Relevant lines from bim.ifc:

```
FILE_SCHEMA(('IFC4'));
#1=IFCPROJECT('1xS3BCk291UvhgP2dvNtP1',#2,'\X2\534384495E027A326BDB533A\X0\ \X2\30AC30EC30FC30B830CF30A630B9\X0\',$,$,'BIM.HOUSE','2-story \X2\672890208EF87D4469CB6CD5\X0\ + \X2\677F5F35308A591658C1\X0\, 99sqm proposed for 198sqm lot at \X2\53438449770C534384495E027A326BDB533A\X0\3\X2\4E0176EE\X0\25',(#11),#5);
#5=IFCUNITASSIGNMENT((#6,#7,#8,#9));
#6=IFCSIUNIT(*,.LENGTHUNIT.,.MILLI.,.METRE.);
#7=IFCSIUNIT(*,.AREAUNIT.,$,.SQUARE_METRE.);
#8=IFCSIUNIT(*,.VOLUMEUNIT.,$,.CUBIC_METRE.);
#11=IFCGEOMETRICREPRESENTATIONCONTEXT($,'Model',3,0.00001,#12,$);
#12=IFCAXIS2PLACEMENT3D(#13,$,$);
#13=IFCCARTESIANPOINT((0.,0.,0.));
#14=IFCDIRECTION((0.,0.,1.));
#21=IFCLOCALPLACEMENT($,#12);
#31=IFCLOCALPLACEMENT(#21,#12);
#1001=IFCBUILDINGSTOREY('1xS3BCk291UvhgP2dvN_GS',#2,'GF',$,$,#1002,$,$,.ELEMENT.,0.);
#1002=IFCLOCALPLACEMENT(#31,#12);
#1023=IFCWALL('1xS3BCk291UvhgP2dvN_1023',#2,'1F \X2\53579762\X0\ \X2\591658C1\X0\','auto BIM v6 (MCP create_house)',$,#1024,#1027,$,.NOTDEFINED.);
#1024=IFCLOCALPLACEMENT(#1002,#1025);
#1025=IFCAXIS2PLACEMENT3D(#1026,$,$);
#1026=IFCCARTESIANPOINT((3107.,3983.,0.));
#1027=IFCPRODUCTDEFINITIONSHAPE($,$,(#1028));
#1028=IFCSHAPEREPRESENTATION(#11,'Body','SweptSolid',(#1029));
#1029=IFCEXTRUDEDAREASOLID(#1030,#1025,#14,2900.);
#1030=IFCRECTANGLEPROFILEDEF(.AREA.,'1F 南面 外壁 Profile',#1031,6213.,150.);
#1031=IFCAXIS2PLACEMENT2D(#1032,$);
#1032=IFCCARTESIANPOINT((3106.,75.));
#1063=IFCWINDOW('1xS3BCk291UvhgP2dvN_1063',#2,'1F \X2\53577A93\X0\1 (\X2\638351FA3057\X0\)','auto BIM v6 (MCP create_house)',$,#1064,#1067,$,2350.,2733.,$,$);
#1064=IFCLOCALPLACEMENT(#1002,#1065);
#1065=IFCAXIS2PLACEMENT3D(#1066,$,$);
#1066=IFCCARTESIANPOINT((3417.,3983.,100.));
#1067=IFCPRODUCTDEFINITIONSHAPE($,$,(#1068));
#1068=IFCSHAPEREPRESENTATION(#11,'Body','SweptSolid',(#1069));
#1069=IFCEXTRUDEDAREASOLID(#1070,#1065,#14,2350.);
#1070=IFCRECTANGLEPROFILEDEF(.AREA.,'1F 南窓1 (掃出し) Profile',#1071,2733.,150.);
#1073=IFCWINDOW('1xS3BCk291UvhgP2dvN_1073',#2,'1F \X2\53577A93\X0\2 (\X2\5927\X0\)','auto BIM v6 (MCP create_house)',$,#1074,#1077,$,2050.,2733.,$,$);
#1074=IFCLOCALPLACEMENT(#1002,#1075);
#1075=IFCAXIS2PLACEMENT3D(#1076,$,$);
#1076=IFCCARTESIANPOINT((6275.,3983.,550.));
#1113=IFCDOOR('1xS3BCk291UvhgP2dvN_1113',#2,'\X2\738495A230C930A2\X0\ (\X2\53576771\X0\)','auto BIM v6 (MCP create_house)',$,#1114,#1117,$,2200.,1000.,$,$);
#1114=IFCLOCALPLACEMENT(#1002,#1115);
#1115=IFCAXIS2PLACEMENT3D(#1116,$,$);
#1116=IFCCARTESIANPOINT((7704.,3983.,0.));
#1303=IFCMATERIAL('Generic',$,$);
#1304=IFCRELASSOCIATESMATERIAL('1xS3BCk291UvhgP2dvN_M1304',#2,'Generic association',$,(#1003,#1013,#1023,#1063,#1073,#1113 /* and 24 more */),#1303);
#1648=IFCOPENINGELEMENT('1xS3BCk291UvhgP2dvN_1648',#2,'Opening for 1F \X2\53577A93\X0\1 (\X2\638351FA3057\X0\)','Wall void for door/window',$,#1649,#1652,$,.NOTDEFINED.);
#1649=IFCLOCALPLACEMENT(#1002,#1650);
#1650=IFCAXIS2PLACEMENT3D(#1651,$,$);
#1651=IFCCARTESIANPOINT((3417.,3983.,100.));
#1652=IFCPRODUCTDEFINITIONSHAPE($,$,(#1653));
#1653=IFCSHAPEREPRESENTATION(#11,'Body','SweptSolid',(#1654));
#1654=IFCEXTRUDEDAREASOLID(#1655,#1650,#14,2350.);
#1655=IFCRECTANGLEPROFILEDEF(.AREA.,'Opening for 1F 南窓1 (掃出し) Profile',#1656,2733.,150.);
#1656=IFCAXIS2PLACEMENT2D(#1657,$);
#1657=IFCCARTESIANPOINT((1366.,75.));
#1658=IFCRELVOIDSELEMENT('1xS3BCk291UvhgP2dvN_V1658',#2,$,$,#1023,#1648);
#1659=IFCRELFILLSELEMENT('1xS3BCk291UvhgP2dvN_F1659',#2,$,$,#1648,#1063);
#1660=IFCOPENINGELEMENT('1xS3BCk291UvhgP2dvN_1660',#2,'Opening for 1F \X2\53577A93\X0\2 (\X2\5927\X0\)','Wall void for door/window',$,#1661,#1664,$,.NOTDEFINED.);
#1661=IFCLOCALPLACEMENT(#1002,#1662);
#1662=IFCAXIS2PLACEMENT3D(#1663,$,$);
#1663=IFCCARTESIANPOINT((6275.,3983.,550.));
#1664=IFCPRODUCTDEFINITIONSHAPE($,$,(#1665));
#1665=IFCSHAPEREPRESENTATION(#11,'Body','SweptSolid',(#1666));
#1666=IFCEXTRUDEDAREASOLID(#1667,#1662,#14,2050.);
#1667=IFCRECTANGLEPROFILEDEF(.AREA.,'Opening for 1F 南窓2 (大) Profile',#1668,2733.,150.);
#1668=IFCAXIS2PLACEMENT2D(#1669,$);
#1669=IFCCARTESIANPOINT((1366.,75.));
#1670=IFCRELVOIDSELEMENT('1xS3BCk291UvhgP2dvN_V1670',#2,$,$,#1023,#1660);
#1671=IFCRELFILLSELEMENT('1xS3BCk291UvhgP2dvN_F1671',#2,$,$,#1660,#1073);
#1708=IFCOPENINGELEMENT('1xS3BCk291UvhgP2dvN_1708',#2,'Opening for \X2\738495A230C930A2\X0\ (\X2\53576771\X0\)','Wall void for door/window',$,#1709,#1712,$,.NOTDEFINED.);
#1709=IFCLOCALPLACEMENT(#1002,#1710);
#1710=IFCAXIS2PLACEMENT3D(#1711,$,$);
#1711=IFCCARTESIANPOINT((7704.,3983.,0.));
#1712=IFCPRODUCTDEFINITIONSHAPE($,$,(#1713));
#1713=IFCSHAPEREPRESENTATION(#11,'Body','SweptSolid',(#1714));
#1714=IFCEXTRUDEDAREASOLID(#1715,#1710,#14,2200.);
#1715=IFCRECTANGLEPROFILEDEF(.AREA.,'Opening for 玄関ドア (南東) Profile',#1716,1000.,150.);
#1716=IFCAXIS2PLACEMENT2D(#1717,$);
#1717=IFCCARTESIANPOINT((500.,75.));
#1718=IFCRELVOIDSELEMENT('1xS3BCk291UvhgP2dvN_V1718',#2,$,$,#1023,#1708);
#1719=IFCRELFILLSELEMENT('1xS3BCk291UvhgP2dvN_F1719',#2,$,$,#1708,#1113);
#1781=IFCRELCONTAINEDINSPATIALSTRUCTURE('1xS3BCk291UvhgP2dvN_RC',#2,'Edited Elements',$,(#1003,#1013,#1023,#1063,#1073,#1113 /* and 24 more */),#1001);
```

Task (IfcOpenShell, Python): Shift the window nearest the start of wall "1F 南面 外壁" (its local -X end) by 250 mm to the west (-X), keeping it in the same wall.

```python
import ifcopenshell
import ifcopenshell.api.geometry
import ifcopenshell.util.placement

model = ifcopenshell.open("bim.ifc")

window = model.by_guid("1xS3BCk291UvhgP2dvN_1063")
opening = window.FillsVoids[0].RelatingOpeningElement
wall = opening.VoidsElements[0].RelatingBuildingElement

wall_matrix = ifcopenshell.util.placement.get_local_placement(wall.ObjectPlacement)
shift = wall_matrix[:3, 0] * -250.0
before = ifcopenshell.util.placement.get_local_placement(window.ObjectPlacement)[:3, 3].copy()

# The window is not placed relative to its opening, so move both.
for product in (opening, window):
    matrix = ifcopenshell.util.placement.get_local_placement(product.ObjectPlacement)
    matrix[:3, 3] += shift
    ifcopenshell.api.geometry.edit_object_placement(model, product=product, matrix=matrix, is_si=False)

after = ifcopenshell.util.placement.get_local_placement(window.ObjectPlacement)[:3, 3]
print("window moved by", (after - before).round(3) + 0.0)

model.write("bim_rev.ifc")
```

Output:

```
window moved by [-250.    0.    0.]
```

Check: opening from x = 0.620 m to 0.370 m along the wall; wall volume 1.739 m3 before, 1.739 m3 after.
